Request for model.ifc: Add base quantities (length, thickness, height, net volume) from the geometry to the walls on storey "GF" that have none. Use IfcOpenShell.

First a look at what the model holds.

```python
import ifcopenshell
import ifcopenshell.util.element
import ifcopenshell.util.unit

model = ifcopenshell.open("model.ifc")
print(model.schema)
for unit_type in ("LENGTHUNIT", "AREAUNIT", "VOLUMEUNIT"):
    print(unit_type, ifcopenshell.util.unit.calculate_unit_scale(model, unit_type))
storey = next(s for s in model.by_type("IfcBuildingStorey") if s.Name == "GF")
walls = [e for e in ifcopenshell.util.element.get_decomposition(storey) if e.is_a("IfcWall")]
for e in sorted(walls, key=lambda e: e.id()):
    print(e.id(), e.is_a(), e.Name, list(ifcopenshell.util.element.get_psets(e, qtos_only=True)), sep=" | ")
```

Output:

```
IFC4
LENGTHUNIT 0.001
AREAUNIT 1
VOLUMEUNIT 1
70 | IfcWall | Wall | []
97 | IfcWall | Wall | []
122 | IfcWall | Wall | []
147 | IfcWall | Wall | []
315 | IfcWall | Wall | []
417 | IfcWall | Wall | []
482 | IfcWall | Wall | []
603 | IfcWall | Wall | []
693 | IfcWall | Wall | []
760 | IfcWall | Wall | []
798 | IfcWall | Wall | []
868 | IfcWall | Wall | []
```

```python
import ifcopenshell
import ifcopenshell.api.pset
import ifcopenshell.geom
import ifcopenshell.util.element
import ifcopenshell.util.shape
import ifcopenshell.util.unit

model = ifcopenshell.open("model.ifc")
unit_scale = ifcopenshell.util.unit.calculate_unit_scale(model)
volume_scale = ifcopenshell.util.unit.calculate_unit_scale(model, "VOLUMEUNIT")
settings = ifcopenshell.geom.settings()

storey = next(s for s in model.by_type("IfcBuildingStorey") if s.Name == "GF")
walls = [e for e in ifcopenshell.util.element.get_decomposition(storey) if e.is_a("IfcWall")]

for e in sorted(walls, key=lambda e: e.id()):
    if ifcopenshell.util.element.get_psets(e, qtos_only=True, should_inherit=False):
        continue
    # Geometry comes back in metres, in the element's own axes.
    shape = ifcopenshell.geom.create_shape(settings, e)
    values = {
        "Length": ifcopenshell.util.shape.get_x(shape.geometry) / unit_scale,
        "Width": ifcopenshell.util.shape.get_y(shape.geometry) / unit_scale,
        "Height": ifcopenshell.util.shape.get_z(shape.geometry) / unit_scale,
        "NetVolume": ifcopenshell.util.shape.get_volume(shape.geometry) / volume_scale,
    }
    qto = ifcopenshell.api.pset.add_qto(model, product=e, name="Qto_WallBaseQuantities")
    ifcopenshell.api.pset.edit_qto(model, qto=qto, properties=values)
    print(e.id(), {k: round(v, 3) for k, v in values.items()})

model.write("model_v2.ifc")
```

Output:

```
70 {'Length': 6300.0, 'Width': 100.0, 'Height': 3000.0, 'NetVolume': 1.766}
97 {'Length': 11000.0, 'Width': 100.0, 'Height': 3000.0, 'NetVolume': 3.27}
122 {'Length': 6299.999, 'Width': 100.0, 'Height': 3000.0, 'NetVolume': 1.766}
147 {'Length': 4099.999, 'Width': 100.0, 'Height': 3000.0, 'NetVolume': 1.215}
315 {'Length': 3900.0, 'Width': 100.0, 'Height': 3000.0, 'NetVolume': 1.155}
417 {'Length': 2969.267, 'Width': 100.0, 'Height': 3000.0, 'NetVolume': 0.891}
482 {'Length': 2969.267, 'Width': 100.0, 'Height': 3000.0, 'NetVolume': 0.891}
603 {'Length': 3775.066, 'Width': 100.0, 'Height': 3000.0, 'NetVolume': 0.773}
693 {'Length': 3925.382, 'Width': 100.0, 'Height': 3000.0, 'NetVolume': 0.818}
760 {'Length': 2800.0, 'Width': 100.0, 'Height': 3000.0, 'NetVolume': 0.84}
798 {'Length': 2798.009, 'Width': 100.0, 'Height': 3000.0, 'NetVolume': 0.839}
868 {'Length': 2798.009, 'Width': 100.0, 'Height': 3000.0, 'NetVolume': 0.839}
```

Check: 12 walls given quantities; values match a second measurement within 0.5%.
